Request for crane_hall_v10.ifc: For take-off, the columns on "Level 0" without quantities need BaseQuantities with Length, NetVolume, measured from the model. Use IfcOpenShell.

First a look at what the model holds.

```python
import ifcopenshell
import ifcopenshell.util.element
import ifcopenshell.util.unit

model = ifcopenshell.open("crane_hall_v10.ifc")
print(model.schema)
for unit_type in ("LENGTHUNIT", "AREAUNIT", "VOLUMEUNIT"):
    print(unit_type, ifcopenshell.util.unit.calculate_unit_scale(model, unit_type))
storey = next(s for s in model.by_type("IfcBuildingStorey") if s.Name == "Level 0")
columns = [e for e in ifcopenshell.util.element.get_decomposition(storey) if e.is_a("IfcColumn")]
for e in sorted(columns, key=lambda e: e.id()):
    print(e.id(), e.is_a(), e.Name, list(ifcopenshell.util.element.get_psets(e, qtos_only=True)), sep=" | ")
```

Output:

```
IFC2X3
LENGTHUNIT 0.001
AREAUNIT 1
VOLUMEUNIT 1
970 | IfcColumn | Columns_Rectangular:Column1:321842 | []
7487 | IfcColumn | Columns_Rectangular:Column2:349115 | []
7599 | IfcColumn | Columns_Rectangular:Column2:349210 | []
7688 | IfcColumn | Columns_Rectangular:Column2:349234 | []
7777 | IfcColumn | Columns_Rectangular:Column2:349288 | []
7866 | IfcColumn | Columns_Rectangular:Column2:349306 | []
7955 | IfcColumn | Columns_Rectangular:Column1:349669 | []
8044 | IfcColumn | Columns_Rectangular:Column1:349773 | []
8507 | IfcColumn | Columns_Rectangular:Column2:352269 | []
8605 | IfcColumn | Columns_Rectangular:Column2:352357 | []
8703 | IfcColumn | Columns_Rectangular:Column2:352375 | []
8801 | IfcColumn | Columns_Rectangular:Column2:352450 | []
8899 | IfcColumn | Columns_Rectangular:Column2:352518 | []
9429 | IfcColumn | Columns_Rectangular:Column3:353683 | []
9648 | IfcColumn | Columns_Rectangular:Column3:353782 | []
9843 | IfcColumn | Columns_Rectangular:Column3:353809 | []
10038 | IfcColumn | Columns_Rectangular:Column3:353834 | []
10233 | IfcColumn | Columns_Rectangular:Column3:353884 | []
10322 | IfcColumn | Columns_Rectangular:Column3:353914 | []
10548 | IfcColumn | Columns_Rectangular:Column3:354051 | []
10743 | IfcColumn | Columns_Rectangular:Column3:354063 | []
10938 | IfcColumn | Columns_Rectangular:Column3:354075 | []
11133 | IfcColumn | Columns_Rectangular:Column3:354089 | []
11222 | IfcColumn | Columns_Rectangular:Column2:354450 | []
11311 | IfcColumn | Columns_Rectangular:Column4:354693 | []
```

```python
import ifcopenshell
import ifcopenshell.api.pset
import ifcopenshell.geom
import ifcopenshell.util.element
import ifcopenshell.util.shape
import ifcopenshell.util.unit

model = ifcopenshell.open("crane_hall_v10.ifc")
unit_scale = ifcopenshell.util.unit.calculate_unit_scale(model)
volume_scale = ifcopenshell.util.unit.calculate_unit_scale(model, "VOLUMEUNIT")
settings = ifcopenshell.geom.settings()

storey = next(s for s in model.by_type("IfcBuildingStorey") if s.Name == "Level 0")
columns = [e for e in ifcopenshell.util.element.get_decomposition(storey) if e.is_a("IfcColumn")]

for e in sorted(columns, key=lambda e: e.id()):
    if ifcopenshell.util.element.get_psets(e, qtos_only=True, should_inherit=False):
        continue
    # Geometry comes back in metres, in the element's own axes.
    shape = ifcopenshell.geom.create_shape(settings, e)
    values = {
        "Length": ifcopenshell.util.shape.get_z(shape.geometry) / unit_scale,
        "NetVolume": ifcopenshell.util.shape.get_volume(shape.geometry) / volume_scale,
    }
    qto = ifcopenshell.api.pset.add_qto(model, product=e, name="BaseQuantities")
    ifcopenshell.api.pset.edit_qto(model, qto=qto, properties=values)
    print(e.id(), {k: round(v, 3) for k, v in values.items()})

model.write("crane_hall_v10_v2.ifc")
```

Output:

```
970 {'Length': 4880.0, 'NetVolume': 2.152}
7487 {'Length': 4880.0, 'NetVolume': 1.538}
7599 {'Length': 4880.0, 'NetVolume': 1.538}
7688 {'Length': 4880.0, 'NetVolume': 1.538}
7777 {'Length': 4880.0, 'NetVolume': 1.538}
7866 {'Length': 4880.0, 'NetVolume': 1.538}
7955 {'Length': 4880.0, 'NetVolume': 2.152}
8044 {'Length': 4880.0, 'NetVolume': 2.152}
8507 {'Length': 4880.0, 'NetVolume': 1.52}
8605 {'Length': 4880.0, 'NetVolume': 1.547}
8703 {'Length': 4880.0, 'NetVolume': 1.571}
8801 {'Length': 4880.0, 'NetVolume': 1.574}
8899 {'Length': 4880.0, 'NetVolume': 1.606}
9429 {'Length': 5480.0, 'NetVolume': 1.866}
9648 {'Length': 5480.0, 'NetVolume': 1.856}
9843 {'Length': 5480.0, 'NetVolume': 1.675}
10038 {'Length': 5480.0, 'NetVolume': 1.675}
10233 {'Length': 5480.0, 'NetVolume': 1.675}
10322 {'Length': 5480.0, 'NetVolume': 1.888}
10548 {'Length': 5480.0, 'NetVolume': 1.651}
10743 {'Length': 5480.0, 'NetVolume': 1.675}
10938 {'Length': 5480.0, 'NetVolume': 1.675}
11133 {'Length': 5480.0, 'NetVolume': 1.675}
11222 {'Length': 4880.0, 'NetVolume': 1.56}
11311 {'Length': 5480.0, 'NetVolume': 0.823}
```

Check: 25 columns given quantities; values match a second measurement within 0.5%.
